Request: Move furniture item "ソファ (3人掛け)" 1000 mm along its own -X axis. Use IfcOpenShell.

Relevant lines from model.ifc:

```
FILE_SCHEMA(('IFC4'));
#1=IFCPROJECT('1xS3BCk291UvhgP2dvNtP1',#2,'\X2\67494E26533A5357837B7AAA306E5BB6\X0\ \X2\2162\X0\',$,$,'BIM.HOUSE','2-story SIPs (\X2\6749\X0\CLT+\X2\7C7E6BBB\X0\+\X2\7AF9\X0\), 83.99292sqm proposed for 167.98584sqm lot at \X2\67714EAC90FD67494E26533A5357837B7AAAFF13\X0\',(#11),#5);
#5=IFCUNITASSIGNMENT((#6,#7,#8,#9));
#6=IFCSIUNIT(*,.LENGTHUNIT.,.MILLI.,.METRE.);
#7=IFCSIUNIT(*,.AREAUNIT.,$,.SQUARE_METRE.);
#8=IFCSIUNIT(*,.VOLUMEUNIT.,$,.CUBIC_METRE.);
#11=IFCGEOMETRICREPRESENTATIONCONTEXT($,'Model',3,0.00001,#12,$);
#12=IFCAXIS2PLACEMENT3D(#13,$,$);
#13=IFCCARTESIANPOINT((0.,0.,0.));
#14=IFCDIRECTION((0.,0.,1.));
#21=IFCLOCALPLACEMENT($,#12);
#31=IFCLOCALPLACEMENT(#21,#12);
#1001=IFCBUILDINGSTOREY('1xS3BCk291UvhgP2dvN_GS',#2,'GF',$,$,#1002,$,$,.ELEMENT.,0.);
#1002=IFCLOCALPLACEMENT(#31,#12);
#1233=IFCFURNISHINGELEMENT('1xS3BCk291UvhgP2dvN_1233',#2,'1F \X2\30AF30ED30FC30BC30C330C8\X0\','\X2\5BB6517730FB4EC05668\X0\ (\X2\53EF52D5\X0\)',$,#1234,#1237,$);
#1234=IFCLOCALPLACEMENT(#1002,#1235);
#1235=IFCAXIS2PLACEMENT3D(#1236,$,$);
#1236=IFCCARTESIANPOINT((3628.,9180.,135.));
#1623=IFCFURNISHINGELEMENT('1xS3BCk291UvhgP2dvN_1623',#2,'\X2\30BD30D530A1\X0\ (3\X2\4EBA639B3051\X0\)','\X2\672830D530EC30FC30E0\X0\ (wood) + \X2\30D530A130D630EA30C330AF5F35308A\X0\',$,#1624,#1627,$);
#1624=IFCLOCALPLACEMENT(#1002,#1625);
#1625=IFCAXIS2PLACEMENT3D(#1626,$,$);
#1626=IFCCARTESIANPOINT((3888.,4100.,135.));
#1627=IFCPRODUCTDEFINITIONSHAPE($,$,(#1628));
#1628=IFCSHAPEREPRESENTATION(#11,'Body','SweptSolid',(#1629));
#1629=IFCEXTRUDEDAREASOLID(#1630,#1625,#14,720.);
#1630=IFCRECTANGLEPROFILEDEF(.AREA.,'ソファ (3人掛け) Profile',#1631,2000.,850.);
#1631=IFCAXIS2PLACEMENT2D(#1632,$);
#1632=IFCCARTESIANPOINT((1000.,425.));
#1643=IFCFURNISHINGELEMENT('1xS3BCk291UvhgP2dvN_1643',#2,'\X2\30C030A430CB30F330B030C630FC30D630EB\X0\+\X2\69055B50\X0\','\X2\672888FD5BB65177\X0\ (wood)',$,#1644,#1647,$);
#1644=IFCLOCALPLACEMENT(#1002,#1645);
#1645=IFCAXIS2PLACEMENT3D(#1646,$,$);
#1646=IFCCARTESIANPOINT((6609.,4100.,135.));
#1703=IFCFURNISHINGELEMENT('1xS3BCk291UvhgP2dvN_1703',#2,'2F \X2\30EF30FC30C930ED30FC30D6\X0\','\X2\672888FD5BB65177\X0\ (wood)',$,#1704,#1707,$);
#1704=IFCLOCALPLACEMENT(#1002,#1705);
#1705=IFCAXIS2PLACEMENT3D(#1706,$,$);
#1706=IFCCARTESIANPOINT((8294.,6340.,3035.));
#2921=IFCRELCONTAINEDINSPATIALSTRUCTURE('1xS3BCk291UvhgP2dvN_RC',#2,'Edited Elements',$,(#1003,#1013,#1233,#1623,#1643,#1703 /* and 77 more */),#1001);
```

```python
import ifcopenshell
import ifcopenshell.api.geometry
import ifcopenshell.util.placement
import ifcopenshell.util.unit

model = ifcopenshell.open("model.ifc")
unit_scale = ifcopenshell.util.unit.calculate_unit_scale(model)

item = model.by_guid("1xS3BCk291UvhgP2dvN_1623")
matrix = ifcopenshell.util.placement.get_local_placement(item.ObjectPlacement)
matrix[:3, 3] -= matrix[:3, 0] * 1 / unit_scale
ifcopenshell.api.geometry.edit_object_placement(model, product=item, matrix=matrix, is_si=False)

print(ifcopenshell.util.placement.get_local_placement(item.ObjectPlacement).round(3) + 0.0)

model.write("model_v2.ifc")
```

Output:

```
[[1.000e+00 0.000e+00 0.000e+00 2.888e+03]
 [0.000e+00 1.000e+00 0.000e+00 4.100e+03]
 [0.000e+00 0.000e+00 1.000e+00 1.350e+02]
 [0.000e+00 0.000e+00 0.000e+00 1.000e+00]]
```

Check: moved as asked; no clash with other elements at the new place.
